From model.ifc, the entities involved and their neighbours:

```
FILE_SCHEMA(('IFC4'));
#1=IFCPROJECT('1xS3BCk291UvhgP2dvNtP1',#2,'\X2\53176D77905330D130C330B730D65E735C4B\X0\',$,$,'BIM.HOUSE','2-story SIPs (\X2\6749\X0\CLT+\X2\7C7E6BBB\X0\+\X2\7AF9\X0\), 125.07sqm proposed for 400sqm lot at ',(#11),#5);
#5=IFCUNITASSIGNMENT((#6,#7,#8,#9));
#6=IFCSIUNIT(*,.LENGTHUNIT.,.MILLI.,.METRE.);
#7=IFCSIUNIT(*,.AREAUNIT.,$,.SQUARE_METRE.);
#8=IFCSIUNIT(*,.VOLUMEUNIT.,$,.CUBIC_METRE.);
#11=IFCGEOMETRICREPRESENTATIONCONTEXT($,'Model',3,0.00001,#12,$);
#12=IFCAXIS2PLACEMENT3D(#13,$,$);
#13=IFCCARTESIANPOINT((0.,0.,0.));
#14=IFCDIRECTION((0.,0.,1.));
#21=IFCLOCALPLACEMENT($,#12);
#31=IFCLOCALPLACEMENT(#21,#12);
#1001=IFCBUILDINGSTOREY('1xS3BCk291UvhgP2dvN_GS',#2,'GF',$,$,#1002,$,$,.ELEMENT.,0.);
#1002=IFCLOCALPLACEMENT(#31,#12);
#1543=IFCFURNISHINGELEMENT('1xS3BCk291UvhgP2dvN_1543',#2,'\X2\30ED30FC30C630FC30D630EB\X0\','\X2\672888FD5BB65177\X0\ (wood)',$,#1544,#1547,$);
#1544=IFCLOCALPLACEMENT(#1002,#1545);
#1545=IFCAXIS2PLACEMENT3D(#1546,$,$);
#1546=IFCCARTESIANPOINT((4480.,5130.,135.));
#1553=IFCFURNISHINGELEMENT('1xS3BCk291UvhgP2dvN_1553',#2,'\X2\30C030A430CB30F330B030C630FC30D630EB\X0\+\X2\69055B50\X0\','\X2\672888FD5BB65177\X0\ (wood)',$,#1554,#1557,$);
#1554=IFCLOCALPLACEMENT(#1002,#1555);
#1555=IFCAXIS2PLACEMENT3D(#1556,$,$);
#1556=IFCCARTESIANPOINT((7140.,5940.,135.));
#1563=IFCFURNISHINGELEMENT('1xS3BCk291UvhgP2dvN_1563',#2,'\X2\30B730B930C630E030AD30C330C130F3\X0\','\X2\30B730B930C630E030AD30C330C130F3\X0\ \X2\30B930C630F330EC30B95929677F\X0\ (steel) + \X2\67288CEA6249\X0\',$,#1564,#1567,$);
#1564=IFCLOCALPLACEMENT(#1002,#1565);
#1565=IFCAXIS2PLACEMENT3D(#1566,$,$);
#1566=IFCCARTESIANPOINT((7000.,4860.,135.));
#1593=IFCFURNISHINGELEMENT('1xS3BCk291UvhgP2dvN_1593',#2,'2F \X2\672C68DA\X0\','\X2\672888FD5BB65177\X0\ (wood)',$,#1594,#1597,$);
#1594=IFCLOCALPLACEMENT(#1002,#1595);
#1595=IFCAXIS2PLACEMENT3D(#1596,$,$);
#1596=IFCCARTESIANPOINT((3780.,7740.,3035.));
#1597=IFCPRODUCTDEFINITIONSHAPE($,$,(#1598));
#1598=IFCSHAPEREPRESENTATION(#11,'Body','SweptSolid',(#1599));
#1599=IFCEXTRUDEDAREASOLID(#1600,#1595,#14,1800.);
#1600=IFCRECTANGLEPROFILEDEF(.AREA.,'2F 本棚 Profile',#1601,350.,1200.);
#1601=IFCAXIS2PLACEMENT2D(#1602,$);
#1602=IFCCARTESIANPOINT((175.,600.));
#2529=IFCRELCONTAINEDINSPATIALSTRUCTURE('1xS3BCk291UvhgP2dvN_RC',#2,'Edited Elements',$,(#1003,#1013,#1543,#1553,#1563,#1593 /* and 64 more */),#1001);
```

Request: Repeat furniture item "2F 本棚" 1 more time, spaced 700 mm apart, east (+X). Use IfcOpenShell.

```python
import numpy as np
import ifcopenshell
import ifcopenshell.api.geometry
import ifcopenshell.api.root
import ifcopenshell.util.element
import ifcopenshell.util.placement
import ifcopenshell.util.unit

model = ifcopenshell.open("model.ifc")
unit_scale = ifcopenshell.util.unit.calculate_unit_scale(model)


def reuse_history(source, copy):
    """copy_class also copies each property set's owner history, people and application; keep the originals."""
    for rel in copy.IsDefinedBy:
        if rel.is_a("IfcRelDefinesByProperties") and (history := rel.RelatingPropertyDefinition.OwnerHistory):
            rel.RelatingPropertyDefinition.OwnerHistory = source.OwnerHistory
            ifcopenshell.util.element.remove_deep2(model, history)


source = model.by_id(1593)
base = ifcopenshell.util.placement.get_local_placement(source.ObjectPlacement)
step = np.array([1.0, 0.0, 0.0]) * 0.7 / unit_scale

for i in range(1, 2):
    copy = ifcopenshell.api.root.copy_class(model, product=source)
    copy.Representation = ifcopenshell.util.element.copy_deep(
        model, source.Representation, exclude=["IfcGeometricRepresentationContext", "IfcRepresentationMap"]
    )
    reuse_history(source, copy)
    matrix = base.copy()
    matrix[:3, 3] += i * step
    print("added at", matrix[:3, 3].round(3) + 0.0)
    ifcopenshell.api.geometry.edit_object_placement(model, product=copy, matrix=matrix, is_si=False)

model.write("model_edited.ifc")
```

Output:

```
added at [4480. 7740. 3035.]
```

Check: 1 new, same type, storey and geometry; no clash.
